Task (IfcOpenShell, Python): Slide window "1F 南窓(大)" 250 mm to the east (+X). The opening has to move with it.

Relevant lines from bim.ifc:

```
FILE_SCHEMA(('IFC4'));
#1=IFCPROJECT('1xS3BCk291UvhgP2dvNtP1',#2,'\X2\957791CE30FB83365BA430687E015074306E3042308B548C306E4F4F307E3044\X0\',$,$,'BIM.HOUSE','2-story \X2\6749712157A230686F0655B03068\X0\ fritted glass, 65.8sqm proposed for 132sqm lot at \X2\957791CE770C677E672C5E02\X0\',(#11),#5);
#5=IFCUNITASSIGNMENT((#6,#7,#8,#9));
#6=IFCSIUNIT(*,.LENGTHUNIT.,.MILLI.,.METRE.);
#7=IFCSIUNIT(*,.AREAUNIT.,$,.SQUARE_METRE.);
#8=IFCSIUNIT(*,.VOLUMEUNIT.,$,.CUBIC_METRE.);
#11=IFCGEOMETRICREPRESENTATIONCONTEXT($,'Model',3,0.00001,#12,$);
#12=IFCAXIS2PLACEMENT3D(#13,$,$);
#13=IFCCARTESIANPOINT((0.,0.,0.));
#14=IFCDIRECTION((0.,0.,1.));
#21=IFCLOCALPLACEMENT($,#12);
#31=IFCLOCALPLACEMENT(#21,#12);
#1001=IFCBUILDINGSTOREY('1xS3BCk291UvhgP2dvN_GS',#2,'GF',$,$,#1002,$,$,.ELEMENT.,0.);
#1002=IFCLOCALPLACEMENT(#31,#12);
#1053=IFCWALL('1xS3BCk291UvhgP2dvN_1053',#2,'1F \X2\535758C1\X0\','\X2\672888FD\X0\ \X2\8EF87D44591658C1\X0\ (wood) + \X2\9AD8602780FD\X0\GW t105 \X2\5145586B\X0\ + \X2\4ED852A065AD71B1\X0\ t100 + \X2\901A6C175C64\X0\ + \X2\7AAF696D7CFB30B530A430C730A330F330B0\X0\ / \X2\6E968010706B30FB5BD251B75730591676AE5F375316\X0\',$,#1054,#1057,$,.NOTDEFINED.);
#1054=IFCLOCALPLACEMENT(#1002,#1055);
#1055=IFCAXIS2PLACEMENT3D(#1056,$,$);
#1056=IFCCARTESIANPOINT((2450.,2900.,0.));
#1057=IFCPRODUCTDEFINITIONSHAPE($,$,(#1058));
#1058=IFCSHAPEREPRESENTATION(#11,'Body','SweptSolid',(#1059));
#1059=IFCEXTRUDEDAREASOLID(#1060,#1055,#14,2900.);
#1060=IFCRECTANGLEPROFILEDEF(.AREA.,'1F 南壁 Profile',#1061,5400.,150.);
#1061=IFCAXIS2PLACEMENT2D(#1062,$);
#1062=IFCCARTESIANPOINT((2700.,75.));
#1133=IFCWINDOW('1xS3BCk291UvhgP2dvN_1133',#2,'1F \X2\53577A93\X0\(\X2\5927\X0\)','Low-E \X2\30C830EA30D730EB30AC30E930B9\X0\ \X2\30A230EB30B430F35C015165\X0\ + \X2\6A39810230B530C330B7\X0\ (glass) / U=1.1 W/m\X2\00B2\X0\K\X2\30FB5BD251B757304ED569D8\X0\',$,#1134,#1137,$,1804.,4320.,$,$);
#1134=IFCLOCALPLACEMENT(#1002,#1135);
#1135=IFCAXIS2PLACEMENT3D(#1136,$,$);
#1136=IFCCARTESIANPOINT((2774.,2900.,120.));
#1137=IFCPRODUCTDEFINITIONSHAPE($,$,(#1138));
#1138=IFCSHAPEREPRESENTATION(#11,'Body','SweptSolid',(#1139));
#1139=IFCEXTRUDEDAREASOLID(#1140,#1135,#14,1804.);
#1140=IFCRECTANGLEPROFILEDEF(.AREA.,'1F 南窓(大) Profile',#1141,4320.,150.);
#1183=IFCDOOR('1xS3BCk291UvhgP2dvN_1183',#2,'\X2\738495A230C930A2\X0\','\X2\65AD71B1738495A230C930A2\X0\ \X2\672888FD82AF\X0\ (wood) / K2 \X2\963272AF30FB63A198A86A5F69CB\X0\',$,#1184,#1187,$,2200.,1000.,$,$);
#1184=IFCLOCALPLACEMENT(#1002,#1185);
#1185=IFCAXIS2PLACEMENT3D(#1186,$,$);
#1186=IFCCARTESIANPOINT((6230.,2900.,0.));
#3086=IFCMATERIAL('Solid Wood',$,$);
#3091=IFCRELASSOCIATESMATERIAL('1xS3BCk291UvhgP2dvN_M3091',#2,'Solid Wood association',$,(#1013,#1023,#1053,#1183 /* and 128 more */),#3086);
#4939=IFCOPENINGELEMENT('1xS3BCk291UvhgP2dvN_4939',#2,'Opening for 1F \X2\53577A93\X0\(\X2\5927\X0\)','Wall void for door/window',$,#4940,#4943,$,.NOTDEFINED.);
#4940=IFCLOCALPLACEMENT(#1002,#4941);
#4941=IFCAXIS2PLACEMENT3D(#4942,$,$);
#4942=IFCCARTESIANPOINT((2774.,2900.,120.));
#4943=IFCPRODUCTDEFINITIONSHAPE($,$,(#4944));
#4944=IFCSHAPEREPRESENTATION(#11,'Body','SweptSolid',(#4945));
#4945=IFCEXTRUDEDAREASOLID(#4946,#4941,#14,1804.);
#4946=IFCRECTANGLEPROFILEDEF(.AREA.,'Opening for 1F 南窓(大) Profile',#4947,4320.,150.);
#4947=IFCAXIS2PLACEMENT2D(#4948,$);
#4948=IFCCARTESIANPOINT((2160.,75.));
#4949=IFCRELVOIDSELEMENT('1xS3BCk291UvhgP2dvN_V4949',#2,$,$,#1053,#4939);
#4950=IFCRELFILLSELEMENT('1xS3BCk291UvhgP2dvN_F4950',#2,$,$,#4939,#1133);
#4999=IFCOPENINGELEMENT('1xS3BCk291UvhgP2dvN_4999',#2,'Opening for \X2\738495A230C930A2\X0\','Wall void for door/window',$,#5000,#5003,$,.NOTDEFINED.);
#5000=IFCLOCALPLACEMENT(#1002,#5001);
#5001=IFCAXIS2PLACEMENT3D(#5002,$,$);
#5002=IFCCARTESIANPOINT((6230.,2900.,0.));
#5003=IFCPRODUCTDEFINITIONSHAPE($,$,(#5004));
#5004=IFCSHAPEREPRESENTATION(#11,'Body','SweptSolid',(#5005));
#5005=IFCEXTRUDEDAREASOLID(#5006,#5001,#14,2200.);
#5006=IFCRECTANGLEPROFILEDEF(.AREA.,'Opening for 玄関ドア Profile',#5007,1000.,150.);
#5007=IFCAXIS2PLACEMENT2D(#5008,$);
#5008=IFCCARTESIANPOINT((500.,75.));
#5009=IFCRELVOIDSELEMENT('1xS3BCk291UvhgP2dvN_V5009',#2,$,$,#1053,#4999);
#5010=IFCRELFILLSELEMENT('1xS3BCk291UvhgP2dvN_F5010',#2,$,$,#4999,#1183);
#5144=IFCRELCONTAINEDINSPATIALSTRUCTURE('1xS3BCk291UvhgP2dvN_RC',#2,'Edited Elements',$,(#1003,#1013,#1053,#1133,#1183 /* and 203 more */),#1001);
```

```python
import ifcopenshell
import ifcopenshell.api.geometry
import ifcopenshell.util.placement
import ifcopenshell.util.unit

model = ifcopenshell.open("bim.ifc")
unit_scale = ifcopenshell.util.unit.calculate_unit_scale(model)

window = model.by_guid("1xS3BCk291UvhgP2dvN_1133")
opening = window.FillsVoids[0].RelatingOpeningElement
wall = opening.VoidsElements[0].RelatingBuildingElement

wall_matrix = ifcopenshell.util.placement.get_local_placement(wall.ObjectPlacement)
shift = wall_matrix[:3, 0] * 0.25 / unit_scale
before = ifcopenshell.util.placement.get_local_placement(window.ObjectPlacement)[:3, 3].copy()

# The window is not placed relative to its opening, so move both.
for product in (opening, window):
    matrix = ifcopenshell.util.placement.get_local_placement(product.ObjectPlacement)
    matrix[:3, 3] += shift
    ifcopenshell.api.geometry.edit_object_placement(model, product=product, matrix=matrix, is_si=False)

after = ifcopenshell.util.placement.get_local_placement(window.ObjectPlacement)[:3, 3]
print("window moved by", (after - before).round(3) + 0.0)

model.write("bim_v2.ifc")
```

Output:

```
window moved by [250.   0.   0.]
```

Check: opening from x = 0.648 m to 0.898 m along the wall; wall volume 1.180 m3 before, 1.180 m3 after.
